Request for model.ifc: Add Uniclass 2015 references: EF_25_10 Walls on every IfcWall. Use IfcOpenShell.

First a look at what the model holds.

```python
import ifcopenshell

model = ifcopenshell.open("model.ifc")
print(model.schema)
print("classifications:", [c.Name for c in model.by_type("IfcClassification")])
for ifc_class in ("IfcDoor", "IfcRoof", "IfcStair", "IfcWall", "IfcWindow"):
    print(ifc_class, len(model.by_type(ifc_class)))
```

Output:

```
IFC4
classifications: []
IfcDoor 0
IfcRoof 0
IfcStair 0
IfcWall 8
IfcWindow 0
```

```python
import ifcopenshell
import ifcopenshell.api.classification

model = ifcopenshell.open("model.ifc")

system = ifcopenshell.api.classification.add_classification(model, classification="Uniclass 2015")

codes = {
    "IfcWall": ("EF_25_10", "Walls"),
}
for ifc_class, (code, name) in codes.items():
    products = model.by_type(ifc_class)
    ifcopenshell.api.classification.add_reference(
        model, products=products, classification=system, identification=code, name=name
    )
    print(code, len(products))

model.write("model_edited.ifc")
```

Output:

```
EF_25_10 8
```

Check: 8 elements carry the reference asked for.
